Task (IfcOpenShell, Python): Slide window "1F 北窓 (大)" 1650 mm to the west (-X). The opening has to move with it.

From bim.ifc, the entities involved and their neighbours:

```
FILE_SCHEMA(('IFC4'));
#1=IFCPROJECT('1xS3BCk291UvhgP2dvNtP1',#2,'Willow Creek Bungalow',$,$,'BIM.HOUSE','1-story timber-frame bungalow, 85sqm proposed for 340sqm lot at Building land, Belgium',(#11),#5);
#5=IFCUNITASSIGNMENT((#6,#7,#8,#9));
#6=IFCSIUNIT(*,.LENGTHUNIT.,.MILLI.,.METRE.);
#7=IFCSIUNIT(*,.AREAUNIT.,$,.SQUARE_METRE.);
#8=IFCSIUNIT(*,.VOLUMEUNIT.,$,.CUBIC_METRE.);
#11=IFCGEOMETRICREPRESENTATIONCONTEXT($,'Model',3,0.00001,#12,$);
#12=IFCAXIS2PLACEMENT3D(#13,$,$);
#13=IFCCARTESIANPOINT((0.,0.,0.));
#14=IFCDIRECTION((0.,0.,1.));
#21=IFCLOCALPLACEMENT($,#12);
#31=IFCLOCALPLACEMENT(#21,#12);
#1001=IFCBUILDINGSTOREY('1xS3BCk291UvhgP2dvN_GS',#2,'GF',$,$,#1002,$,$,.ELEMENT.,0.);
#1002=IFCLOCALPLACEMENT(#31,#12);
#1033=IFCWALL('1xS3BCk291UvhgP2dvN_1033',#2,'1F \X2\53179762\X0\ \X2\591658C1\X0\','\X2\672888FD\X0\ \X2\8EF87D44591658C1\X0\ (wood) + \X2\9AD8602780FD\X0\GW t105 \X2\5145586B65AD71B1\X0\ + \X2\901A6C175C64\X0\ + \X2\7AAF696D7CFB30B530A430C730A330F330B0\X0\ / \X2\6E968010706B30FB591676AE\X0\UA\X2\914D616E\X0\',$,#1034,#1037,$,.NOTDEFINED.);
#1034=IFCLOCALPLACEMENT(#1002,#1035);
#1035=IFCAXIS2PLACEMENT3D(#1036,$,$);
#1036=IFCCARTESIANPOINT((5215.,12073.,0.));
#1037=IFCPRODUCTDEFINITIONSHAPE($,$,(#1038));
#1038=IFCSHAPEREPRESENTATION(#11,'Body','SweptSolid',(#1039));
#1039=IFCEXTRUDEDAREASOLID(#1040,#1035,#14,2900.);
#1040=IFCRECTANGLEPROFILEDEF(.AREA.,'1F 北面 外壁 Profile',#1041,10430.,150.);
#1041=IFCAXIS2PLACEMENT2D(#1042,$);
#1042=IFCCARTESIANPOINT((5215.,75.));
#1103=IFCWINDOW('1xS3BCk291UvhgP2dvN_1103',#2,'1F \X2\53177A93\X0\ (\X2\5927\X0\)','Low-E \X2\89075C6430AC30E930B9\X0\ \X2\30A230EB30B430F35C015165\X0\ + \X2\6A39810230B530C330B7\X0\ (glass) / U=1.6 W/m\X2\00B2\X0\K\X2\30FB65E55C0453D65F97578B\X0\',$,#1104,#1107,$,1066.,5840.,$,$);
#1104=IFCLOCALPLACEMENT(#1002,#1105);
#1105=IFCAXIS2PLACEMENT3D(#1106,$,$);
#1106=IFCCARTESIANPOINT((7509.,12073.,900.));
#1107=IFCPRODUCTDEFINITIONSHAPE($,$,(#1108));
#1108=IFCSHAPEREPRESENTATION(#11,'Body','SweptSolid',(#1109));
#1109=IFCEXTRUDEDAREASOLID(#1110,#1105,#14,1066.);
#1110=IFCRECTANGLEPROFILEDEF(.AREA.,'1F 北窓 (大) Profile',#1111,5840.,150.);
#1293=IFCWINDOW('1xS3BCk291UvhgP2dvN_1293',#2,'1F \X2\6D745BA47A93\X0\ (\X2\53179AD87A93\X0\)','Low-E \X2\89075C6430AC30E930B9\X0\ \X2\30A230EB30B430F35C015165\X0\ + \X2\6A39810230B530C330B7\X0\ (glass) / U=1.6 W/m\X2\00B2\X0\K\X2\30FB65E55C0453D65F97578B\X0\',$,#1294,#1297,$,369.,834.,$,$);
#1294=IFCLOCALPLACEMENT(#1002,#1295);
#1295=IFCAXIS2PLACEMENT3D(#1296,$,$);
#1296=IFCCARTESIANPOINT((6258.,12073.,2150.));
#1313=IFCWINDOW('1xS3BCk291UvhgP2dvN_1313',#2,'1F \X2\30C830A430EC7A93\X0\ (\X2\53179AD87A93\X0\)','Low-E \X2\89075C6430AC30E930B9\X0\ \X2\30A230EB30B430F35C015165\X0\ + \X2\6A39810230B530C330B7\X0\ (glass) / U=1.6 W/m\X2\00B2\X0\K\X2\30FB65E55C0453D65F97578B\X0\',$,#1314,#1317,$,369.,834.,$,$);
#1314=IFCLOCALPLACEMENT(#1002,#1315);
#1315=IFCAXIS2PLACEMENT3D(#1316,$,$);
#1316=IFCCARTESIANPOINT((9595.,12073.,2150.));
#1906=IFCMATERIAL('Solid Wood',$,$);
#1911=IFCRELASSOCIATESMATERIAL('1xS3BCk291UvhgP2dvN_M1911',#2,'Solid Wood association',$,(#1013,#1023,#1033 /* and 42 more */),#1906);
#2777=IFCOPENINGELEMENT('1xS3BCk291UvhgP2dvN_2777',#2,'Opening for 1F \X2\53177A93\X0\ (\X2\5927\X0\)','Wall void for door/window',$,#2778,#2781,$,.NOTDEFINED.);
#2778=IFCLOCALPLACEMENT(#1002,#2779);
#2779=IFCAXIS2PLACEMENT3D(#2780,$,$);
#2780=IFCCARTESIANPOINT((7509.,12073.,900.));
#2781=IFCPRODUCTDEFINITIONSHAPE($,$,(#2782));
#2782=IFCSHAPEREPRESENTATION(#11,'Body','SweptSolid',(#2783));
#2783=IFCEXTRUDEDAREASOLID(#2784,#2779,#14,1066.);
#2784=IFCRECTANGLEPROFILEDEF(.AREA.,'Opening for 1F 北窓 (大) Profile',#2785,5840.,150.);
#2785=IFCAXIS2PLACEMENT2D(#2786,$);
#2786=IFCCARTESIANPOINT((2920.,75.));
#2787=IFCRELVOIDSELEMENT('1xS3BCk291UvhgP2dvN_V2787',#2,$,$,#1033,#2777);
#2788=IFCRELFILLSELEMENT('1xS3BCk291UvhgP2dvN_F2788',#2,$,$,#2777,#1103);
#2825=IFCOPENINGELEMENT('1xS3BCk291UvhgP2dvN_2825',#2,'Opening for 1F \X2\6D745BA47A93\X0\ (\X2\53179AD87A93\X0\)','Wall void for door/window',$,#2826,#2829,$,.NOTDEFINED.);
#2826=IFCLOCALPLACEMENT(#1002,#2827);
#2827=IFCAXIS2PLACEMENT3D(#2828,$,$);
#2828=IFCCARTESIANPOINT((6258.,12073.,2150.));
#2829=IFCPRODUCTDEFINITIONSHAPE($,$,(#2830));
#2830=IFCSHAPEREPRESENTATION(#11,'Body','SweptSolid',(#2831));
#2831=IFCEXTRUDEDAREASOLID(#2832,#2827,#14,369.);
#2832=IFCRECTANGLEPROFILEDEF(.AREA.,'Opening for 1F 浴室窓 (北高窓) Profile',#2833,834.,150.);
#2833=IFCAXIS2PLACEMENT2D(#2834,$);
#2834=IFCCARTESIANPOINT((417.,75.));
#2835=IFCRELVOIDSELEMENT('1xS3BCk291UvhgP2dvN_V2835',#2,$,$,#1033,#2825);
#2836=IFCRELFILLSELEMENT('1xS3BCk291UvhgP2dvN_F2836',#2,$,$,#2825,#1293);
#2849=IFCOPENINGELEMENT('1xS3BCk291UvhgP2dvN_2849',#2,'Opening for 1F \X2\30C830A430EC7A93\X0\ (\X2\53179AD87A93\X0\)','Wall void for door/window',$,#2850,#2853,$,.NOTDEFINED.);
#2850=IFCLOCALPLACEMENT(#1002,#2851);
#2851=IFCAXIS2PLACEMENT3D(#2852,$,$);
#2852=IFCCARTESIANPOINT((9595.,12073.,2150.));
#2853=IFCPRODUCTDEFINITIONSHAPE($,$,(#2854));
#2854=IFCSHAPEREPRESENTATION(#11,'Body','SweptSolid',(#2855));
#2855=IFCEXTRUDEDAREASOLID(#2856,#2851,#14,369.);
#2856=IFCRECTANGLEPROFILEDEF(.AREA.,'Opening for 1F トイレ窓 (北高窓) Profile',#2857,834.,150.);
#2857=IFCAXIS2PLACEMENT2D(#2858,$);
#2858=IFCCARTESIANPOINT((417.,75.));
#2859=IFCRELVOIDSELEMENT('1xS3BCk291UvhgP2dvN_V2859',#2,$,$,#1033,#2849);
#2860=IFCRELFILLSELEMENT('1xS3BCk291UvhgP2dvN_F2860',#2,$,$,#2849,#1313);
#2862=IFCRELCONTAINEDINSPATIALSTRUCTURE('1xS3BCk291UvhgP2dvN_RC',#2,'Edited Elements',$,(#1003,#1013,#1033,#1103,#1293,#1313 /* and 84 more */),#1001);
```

```python
import ifcopenshell
import ifcopenshell.api.geometry
import ifcopenshell.util.placement
import ifcopenshell.util.unit

model = ifcopenshell.open("bim.ifc")
unit_scale = ifcopenshell.util.unit.calculate_unit_scale(model)

window = model.by_guid("1xS3BCk291UvhgP2dvN_1103")
opening = window.FillsVoids[0].RelatingOpeningElement
wall = opening.VoidsElements[0].RelatingBuildingElement

wall_matrix = ifcopenshell.util.placement.get_local_placement(wall.ObjectPlacement)
shift = wall_matrix[:3, 0] * -1.65 / unit_scale
before = ifcopenshell.util.placement.get_local_placement(window.ObjectPlacement)[:3, 3].copy()

# The window is not placed relative to its opening, so move both.
for product in (opening, window):
    matrix = ifcopenshell.util.placement.get_local_placement(product.ObjectPlacement)
    matrix[:3, 3] += shift
    ifcopenshell.api.geometry.edit_object_placement(model, product=product, matrix=matrix, is_si=False)

after = ifcopenshell.util.placement.get_local_placement(window.ObjectPlacement)[:3, 3]
print("window moved by", (after - before).round(3) + 0.0)

model.write("bim-out.ifc")
```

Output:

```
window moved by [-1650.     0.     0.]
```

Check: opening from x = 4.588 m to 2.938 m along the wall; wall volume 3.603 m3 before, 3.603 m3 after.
